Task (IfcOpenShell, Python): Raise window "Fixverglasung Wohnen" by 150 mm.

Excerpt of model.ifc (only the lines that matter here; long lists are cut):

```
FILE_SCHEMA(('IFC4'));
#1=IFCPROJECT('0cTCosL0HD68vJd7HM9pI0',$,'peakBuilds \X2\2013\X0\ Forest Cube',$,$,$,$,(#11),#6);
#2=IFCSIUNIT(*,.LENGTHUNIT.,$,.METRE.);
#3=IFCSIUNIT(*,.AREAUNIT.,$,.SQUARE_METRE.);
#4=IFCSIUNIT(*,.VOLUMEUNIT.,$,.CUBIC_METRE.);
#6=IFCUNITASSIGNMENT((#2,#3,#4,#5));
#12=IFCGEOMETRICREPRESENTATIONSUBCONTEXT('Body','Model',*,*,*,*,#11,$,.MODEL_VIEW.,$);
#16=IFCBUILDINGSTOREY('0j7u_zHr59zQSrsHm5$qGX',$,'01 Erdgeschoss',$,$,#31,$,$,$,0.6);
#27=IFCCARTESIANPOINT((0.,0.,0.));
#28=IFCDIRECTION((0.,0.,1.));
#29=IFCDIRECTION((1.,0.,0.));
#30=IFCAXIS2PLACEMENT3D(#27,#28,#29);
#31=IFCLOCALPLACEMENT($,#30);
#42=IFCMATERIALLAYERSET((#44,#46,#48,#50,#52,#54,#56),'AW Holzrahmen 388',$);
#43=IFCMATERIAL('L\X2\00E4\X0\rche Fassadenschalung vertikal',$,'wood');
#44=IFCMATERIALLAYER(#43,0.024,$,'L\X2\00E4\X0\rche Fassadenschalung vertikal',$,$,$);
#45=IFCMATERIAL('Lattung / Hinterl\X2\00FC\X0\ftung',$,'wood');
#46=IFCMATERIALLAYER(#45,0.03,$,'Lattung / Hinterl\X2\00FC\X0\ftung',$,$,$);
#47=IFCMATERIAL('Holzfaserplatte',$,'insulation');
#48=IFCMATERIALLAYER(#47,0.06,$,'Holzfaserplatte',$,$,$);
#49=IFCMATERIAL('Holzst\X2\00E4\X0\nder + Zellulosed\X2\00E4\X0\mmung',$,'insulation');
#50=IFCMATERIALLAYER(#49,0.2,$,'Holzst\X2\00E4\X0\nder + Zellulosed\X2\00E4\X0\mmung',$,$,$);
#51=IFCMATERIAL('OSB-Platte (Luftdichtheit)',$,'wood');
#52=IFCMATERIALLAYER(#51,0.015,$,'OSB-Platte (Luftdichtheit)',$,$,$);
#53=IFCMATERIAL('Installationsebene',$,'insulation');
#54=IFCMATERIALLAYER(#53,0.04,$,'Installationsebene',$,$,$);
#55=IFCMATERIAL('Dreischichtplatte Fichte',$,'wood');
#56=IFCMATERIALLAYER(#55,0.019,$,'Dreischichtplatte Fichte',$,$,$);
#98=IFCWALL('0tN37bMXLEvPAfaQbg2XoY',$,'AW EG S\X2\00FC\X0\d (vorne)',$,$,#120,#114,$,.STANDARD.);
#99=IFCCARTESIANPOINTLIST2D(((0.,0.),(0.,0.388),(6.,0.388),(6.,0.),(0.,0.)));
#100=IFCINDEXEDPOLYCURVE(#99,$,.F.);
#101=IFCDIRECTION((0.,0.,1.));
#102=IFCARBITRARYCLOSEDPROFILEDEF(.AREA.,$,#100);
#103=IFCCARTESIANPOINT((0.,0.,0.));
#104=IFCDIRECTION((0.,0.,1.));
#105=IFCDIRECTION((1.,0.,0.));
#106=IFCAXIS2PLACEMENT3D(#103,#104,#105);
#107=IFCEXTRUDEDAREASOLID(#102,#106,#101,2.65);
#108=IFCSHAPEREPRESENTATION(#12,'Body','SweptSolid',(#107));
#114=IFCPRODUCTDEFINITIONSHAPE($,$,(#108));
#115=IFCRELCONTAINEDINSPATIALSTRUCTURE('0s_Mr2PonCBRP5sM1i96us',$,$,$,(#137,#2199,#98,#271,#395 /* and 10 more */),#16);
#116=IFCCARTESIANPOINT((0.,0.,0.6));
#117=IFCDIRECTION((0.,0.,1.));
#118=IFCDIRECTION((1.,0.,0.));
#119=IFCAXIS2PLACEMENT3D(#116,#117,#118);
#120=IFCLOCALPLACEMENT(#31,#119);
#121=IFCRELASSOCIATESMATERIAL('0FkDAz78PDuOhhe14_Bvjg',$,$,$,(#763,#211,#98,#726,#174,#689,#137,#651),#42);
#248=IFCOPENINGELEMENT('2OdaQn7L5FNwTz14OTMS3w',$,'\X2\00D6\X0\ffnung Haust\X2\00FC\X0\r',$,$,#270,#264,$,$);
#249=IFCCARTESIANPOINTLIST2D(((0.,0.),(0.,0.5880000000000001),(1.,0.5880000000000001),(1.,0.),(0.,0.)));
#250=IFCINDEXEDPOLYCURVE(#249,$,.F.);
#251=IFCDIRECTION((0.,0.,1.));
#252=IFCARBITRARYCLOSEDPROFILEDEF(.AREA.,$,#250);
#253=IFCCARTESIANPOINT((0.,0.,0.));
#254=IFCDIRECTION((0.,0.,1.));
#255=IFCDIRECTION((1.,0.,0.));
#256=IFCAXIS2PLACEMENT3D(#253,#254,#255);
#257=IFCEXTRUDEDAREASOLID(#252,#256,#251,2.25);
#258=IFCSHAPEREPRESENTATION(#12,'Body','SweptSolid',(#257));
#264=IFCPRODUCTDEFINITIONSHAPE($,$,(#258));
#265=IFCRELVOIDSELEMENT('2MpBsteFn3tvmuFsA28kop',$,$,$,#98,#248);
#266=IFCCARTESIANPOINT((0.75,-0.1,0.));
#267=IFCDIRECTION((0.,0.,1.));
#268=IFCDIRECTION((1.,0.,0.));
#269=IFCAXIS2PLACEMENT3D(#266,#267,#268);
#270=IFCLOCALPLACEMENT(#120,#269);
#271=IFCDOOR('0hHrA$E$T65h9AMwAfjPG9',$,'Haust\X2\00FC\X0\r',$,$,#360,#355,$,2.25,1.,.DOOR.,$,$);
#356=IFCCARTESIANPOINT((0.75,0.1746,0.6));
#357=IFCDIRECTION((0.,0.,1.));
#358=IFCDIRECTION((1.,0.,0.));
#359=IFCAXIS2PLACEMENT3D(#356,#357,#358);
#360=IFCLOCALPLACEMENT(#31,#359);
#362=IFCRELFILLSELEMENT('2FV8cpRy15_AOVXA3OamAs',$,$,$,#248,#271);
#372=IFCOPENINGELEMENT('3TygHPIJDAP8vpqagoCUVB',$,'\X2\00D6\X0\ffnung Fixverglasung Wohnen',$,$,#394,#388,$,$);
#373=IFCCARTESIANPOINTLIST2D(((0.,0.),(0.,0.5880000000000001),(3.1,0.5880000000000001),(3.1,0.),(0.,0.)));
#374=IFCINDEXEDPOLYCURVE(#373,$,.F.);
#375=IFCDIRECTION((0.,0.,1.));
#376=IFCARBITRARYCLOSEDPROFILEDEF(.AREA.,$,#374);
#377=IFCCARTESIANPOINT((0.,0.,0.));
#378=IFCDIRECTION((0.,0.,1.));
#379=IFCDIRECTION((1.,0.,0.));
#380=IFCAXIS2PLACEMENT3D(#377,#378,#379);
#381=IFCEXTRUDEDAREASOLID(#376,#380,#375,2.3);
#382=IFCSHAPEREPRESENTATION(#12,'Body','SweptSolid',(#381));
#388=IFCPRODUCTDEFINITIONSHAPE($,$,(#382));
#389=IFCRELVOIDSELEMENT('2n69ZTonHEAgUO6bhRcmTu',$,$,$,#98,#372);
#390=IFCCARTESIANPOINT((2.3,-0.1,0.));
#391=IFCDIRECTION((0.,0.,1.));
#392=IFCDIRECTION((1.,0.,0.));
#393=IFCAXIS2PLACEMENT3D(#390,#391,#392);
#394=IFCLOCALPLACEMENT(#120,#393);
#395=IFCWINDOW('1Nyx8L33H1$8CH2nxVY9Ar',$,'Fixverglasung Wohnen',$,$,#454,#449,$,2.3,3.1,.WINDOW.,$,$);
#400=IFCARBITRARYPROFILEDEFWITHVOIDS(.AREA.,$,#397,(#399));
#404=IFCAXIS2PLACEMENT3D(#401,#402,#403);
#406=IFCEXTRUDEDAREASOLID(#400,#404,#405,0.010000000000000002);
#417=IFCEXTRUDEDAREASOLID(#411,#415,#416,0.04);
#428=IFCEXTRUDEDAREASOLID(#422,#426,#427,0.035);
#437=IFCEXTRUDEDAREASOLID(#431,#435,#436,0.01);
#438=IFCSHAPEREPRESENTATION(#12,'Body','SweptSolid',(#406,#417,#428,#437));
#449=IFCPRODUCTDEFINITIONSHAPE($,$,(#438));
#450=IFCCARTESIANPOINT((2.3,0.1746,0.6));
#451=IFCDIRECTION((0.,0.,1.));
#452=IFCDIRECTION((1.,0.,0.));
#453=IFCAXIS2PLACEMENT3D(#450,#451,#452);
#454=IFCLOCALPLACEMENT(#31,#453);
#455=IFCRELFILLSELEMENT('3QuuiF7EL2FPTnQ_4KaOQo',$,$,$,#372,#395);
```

```python
import numpy as np
import ifcopenshell
import ifcopenshell.api.geometry
import ifcopenshell.util.placement
import ifcopenshell.util.unit

model = ifcopenshell.open("model.ifc")
unit_scale = ifcopenshell.util.unit.calculate_unit_scale(model)

window = model.by_guid("1Nyx8L33H1$8CH2nxVY9Ar")
opening = window.FillsVoids[0].RelatingOpeningElement
dz = 0.15 / unit_scale

shift = np.array([0.0, 0.0, dz])
# The window is not placed relative to its opening, so move both.
for product in (opening, window):
    matrix = ifcopenshell.util.placement.get_local_placement(product.ObjectPlacement)
    matrix[:3, 3] += shift
    ifcopenshell.api.geometry.edit_object_placement(model, product=product, matrix=matrix, is_si=False)

print(f"moved by {dz * unit_scale:+.3f} m")

model.write("model_updated.ifc")
```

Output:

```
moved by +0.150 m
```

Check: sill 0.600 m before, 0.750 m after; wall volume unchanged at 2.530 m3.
